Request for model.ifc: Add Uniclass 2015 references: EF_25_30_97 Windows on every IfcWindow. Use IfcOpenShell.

First a look at what the model holds.

```python
import ifcopenshell

model = ifcopenshell.open("model.ifc")
print(model.schema)
print("classifications:", [c.Name for c in model.by_type("IfcClassification")])
for ifc_class in ("IfcDoor", "IfcRoof", "IfcStair", "IfcWall", "IfcWindow"):
    print(ifc_class, len(model.by_type(ifc_class)))
```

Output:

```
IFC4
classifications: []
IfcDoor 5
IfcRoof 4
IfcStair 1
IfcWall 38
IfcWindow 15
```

```python
import ifcopenshell
import ifcopenshell.api.classification

model = ifcopenshell.open("model.ifc")

system = ifcopenshell.api.classification.add_classification(model, classification="Uniclass 2015")

codes = {
    "IfcWindow": ("EF_25_30_97", "Windows"),
}
for ifc_class, (code, name) in codes.items():
    products = model.by_type(ifc_class)
    ifcopenshell.api.classification.add_reference(
        model, products=products, classification=system, identification=code, name=name
    )
    print(code, len(products))

model.write("model_edited.ifc")
```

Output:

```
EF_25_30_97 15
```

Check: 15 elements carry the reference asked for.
